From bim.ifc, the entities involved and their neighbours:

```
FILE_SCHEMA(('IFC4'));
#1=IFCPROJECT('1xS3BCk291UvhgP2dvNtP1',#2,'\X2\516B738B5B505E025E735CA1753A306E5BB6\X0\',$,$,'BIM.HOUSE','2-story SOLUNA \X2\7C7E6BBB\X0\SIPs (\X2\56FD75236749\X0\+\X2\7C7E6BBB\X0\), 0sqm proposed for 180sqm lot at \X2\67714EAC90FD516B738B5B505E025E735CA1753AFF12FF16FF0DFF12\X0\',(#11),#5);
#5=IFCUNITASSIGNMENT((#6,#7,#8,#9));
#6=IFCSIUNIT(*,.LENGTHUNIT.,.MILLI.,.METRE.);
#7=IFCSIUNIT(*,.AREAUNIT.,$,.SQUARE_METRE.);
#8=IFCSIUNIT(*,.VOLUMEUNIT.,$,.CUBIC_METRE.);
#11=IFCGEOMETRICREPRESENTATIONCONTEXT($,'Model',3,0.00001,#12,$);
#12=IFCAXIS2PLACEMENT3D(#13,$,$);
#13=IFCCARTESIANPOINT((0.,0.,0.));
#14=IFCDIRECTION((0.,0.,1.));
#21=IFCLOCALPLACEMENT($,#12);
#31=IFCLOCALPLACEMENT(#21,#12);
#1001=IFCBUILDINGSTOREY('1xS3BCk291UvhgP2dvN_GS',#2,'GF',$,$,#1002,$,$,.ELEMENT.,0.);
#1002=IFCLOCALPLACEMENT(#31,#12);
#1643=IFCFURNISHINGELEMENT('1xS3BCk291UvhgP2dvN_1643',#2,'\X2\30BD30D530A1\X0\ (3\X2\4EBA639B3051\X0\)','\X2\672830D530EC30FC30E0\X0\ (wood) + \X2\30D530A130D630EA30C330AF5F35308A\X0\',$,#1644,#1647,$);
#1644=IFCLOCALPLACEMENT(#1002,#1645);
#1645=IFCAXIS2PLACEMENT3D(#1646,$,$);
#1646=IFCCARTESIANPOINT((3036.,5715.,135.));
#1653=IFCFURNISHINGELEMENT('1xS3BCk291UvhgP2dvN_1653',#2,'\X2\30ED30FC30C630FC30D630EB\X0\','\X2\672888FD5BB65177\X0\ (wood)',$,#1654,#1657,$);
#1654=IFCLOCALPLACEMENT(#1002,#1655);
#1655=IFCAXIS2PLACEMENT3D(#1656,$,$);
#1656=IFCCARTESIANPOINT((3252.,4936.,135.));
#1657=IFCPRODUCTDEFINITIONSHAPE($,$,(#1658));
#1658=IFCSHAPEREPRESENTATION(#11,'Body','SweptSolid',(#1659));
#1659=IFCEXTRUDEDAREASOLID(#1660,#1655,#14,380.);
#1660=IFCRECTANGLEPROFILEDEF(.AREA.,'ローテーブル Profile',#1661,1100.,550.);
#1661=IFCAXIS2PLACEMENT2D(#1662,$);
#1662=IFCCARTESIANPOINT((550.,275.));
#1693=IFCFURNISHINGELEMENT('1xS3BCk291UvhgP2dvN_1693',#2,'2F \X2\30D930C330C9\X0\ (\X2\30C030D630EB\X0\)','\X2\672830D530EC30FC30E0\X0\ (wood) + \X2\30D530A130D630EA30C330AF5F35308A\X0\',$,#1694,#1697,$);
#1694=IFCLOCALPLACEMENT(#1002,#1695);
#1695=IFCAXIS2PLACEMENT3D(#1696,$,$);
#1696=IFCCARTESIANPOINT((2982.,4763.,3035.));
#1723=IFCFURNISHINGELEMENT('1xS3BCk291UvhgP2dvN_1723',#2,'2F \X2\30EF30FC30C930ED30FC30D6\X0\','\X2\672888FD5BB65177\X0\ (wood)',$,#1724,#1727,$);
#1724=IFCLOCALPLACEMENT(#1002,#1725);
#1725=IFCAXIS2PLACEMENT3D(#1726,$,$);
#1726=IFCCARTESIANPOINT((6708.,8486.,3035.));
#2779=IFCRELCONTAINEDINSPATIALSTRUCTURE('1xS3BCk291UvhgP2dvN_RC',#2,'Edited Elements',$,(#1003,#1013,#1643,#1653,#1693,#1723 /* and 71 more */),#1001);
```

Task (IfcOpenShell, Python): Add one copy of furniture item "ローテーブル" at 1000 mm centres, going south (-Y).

```python
import numpy as np
import ifcopenshell
import ifcopenshell.api.geometry
import ifcopenshell.api.root
import ifcopenshell.util.element
import ifcopenshell.util.placement

model = ifcopenshell.open("bim.ifc")


def reuse_history(source, copy):
    """copy_class also copies each property set's owner history, people and application; keep the originals."""
    for rel in copy.IsDefinedBy:
        if rel.is_a("IfcRelDefinesByProperties") and (history := rel.RelatingPropertyDefinition.OwnerHistory):
            rel.RelatingPropertyDefinition.OwnerHistory = source.OwnerHistory
            ifcopenshell.util.element.remove_deep2(model, history)


source = model.by_id(1653)
base = ifcopenshell.util.placement.get_local_placement(source.ObjectPlacement)
step = np.array([0.0, -1.0, 0.0]) * 1000.0

for i in range(1, 2):
    copy = ifcopenshell.api.root.copy_class(model, product=source)
    copy.Representation = ifcopenshell.util.element.copy_deep(
        model, source.Representation, exclude=["IfcGeometricRepresentationContext", "IfcRepresentationMap"]
    )
    reuse_history(source, copy)
    matrix = base.copy()
    matrix[:3, 3] += i * step
    print("added at", matrix[:3, 3].round(3) + 0.0)
    ifcopenshell.api.geometry.edit_object_placement(model, product=copy, matrix=matrix, is_si=False)

model.write("bim_edited.ifc")
```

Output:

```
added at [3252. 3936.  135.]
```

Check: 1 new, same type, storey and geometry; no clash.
